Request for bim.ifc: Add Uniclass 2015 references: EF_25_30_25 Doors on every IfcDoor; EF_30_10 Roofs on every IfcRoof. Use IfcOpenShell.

First a look at what the model holds.

```python
import ifcopenshell

model = ifcopenshell.open("bim.ifc")
print(model.schema)
print("classifications:", [c.Name for c in model.by_type("IfcClassification")])
for ifc_class in ("IfcDoor", "IfcRoof", "IfcStair", "IfcWall", "IfcWindow"):
    print(ifc_class, len(model.by_type(ifc_class)))
```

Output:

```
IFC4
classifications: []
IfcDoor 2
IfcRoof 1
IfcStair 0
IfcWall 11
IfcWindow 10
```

```python
import ifcopenshell
import ifcopenshell.api.classification

model = ifcopenshell.open("bim.ifc")

system = ifcopenshell.api.classification.add_classification(model, classification="Uniclass 2015")

codes = {
    "IfcDoor": ("EF_25_30_25", "Doors"),
    "IfcRoof": ("EF_30_10", "Roofs"),
}
for ifc_class, (code, name) in codes.items():
    products = model.by_type(ifc_class)
    ifcopenshell.api.classification.add_reference(
        model, products=products, classification=system, identification=code, name=name
    )
    print(code, len(products))

model.write("bim-out.ifc")
```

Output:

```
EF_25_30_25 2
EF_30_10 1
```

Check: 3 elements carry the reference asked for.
